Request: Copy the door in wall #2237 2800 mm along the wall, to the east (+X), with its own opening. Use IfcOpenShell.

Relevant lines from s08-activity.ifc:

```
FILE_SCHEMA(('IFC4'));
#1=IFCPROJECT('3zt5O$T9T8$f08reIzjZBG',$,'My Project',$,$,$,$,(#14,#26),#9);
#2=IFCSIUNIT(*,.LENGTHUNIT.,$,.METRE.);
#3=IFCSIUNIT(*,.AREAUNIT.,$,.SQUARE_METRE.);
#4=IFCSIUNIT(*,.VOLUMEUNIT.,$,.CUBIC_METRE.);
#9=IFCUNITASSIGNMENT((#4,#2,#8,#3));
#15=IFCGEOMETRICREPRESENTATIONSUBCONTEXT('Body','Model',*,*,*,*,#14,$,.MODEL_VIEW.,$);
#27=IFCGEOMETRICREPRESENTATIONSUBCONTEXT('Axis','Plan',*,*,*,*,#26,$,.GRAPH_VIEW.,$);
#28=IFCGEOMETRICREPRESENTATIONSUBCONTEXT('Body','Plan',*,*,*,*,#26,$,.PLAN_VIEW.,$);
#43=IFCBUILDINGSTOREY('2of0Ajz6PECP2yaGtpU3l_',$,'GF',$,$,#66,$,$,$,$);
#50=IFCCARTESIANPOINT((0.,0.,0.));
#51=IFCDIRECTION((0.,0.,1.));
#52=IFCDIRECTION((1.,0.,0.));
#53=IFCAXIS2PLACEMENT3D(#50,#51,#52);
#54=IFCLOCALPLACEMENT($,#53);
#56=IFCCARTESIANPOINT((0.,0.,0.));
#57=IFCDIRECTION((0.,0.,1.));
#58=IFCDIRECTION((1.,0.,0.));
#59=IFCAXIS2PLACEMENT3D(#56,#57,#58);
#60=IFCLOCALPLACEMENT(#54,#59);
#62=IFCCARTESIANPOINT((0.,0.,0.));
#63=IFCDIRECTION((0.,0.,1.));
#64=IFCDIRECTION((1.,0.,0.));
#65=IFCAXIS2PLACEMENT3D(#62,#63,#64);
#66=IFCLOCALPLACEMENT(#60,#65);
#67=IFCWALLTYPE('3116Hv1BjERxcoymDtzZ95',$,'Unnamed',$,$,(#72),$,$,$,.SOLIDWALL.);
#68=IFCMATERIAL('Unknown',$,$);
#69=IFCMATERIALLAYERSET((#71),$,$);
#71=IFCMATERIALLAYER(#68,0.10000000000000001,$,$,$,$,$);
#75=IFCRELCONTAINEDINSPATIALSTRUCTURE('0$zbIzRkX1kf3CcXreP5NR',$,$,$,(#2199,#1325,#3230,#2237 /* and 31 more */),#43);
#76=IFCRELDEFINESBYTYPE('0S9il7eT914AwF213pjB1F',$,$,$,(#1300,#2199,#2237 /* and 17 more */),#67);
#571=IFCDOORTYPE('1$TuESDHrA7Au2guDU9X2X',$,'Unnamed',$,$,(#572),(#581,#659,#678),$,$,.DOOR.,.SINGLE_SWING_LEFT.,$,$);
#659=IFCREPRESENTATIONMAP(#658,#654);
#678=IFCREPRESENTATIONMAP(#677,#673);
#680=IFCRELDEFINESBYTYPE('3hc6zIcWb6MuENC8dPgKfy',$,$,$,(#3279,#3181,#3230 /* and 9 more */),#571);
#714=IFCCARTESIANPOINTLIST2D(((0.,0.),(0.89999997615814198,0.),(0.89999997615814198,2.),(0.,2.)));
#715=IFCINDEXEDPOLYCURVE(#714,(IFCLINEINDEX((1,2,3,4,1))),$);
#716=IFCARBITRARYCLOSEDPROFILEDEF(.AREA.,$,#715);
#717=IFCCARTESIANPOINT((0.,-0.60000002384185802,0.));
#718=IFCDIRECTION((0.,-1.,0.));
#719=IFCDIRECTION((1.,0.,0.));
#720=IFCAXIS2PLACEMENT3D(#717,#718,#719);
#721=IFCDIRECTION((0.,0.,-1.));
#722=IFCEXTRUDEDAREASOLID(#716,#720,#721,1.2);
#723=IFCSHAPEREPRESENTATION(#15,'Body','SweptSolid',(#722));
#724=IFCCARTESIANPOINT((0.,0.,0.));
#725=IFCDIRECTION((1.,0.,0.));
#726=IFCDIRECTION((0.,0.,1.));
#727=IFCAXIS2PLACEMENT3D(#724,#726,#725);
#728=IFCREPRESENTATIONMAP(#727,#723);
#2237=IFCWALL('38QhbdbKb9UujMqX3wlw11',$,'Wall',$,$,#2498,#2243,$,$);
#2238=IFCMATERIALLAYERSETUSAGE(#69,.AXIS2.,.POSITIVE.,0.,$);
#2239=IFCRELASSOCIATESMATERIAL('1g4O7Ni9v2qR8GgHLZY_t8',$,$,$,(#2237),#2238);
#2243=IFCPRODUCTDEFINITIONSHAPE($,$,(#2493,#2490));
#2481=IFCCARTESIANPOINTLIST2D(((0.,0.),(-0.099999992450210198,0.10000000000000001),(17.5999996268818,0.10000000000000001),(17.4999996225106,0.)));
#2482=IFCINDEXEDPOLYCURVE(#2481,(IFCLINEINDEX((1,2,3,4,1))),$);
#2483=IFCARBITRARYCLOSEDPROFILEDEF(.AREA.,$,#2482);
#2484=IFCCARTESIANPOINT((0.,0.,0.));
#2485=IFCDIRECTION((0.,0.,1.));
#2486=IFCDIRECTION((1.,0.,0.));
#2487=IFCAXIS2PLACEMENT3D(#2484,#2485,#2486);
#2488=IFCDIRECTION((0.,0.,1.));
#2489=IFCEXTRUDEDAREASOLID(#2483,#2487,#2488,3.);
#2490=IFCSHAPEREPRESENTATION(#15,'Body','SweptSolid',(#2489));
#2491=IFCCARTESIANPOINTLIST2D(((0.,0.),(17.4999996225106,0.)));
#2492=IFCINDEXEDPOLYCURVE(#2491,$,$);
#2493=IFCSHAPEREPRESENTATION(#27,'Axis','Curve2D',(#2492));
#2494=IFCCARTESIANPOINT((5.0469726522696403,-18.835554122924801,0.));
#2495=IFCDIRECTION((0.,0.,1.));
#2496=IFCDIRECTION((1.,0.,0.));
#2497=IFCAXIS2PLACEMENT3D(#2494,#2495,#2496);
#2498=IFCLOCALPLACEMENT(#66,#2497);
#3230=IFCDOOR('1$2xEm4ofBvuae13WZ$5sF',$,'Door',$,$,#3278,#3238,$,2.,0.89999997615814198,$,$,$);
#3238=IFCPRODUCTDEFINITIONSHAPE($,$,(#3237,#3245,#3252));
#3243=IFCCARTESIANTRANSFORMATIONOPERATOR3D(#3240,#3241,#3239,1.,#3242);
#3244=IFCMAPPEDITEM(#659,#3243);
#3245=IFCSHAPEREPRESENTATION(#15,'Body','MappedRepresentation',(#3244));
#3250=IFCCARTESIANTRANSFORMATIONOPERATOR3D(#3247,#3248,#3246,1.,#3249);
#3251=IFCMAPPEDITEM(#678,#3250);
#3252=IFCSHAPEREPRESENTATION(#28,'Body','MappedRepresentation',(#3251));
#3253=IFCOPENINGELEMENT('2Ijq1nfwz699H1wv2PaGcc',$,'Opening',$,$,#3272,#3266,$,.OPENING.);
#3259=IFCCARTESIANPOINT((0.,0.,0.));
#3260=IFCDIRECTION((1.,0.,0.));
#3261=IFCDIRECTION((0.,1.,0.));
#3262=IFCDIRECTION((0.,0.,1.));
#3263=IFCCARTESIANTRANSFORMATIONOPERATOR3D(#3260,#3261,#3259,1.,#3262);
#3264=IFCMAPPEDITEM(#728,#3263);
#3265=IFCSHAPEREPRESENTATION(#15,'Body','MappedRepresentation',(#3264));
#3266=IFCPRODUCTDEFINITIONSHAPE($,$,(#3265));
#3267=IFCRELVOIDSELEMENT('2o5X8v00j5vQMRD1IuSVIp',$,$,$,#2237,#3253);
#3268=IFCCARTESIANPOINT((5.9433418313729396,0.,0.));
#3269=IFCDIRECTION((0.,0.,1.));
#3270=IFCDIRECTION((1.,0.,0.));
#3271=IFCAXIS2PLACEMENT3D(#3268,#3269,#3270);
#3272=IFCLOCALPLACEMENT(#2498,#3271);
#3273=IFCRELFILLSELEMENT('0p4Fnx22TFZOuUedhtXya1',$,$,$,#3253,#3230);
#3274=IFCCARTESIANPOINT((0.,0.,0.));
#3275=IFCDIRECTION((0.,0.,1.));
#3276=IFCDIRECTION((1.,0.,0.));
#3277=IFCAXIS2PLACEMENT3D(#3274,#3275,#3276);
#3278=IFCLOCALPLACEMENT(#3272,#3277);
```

```python
import ifcopenshell
import ifcopenshell.api.feature
import ifcopenshell.api.geometry
import ifcopenshell.api.root
import ifcopenshell.geom
import ifcopenshell.util.element
import ifcopenshell.util.placement
import ifcopenshell.util.shape

model = ifcopenshell.open("s08-activity.ifc")
settings = ifcopenshell.geom.settings()


def volume(element):
    """Net volume in cubic metres, openings subtracted."""
    shape = ifcopenshell.geom.create_shape(settings, element)
    return ifcopenshell.util.shape.get_volume(shape.geometry)


door = model.by_guid("1$2xEm4ofBvuae13WZ$5sF")
opening = door.FillsVoids[0].RelatingOpeningElement
wall = opening.VoidsElements[0].RelatingBuildingElement
before = volume(wall)
shift = ifcopenshell.util.placement.get_local_placement(wall.ObjectPlacement)[:3, 0] * 2.8

# copy_class copies the void relationship, type, container and properties, but no geometry.
new_opening = ifcopenshell.api.root.copy_class(model, product=opening)
new_opening.Representation = ifcopenshell.util.element.copy_deep(
    model, opening.Representation, exclude=["IfcGeometricRepresentationContext", "IfcRepresentationMap"]
)
new_door = ifcopenshell.api.root.copy_class(model, product=door)
new_door.Representation = ifcopenshell.util.element.copy_deep(
    model, door.Representation, exclude=["IfcGeometricRepresentationContext", "IfcRepresentationMap"]
)
ifcopenshell.api.feature.add_filling(model, opening=new_opening, element=new_door)

for old, new in ((opening, new_opening), (door, new_door)):
    matrix = ifcopenshell.util.placement.get_local_placement(old.ObjectPlacement)
    matrix[:3, 3] += shift
    ifcopenshell.api.geometry.edit_object_placement(model, product=new, matrix=matrix, is_si=False)

after = volume(wall)

print(f"wall volume {before:.3f} -> {after:.3f} m3")

model.write("s08-activity_rev.ifc")
```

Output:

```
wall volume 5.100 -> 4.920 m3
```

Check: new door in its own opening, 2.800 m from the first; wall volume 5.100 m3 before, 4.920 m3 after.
